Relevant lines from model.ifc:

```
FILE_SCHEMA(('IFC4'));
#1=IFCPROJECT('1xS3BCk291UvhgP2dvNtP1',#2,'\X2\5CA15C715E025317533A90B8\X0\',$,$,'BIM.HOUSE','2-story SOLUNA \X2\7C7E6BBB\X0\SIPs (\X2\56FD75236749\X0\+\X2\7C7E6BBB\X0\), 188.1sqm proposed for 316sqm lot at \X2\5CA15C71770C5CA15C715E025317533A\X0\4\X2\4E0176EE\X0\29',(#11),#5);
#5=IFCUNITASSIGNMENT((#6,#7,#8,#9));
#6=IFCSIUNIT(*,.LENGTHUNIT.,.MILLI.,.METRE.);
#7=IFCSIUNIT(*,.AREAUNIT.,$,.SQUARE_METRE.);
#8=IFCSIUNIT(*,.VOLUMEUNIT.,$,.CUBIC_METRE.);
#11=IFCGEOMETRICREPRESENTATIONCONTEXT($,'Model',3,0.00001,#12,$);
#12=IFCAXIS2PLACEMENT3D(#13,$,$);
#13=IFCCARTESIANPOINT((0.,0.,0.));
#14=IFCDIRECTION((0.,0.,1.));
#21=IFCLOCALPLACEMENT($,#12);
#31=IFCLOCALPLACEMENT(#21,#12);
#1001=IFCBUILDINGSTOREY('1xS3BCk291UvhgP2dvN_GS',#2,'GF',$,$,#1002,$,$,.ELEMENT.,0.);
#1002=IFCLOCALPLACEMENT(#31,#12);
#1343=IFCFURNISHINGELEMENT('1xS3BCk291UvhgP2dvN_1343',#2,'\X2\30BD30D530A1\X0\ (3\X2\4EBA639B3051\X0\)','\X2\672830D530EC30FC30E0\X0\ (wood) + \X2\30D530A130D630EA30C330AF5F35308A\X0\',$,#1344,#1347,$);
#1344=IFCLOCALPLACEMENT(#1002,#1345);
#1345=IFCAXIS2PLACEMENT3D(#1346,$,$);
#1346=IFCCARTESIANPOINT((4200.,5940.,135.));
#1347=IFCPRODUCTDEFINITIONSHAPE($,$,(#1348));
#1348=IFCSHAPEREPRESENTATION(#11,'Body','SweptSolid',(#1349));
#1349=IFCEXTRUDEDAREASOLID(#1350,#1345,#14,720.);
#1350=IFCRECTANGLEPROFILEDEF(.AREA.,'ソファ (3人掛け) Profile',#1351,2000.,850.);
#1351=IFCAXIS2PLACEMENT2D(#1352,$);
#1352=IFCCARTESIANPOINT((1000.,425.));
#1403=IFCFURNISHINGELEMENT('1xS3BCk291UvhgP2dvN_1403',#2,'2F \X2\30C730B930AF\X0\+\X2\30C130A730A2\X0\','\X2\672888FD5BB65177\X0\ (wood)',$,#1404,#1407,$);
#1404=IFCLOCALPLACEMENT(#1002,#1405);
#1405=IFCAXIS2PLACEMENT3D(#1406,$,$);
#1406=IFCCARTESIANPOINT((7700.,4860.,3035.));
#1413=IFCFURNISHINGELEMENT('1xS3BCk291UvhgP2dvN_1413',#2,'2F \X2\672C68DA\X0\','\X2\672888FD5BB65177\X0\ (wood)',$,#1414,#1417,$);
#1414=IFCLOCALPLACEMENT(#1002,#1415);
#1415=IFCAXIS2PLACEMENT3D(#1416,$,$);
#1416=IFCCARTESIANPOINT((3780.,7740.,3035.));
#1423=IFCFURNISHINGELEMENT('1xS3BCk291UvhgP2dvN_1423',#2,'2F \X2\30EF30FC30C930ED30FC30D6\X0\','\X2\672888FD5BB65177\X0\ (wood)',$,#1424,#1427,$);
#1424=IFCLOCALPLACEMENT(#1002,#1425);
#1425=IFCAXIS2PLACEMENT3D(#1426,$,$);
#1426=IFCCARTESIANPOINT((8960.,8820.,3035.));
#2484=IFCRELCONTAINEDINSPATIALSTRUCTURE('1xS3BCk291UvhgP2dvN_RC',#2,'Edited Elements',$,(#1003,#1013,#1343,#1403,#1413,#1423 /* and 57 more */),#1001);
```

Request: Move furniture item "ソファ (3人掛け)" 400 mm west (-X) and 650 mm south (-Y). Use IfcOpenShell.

```python
import ifcopenshell
import ifcopenshell.api.geometry
import ifcopenshell.util.placement
import ifcopenshell.util.unit

model = ifcopenshell.open("model.ifc")
unit_scale = ifcopenshell.util.unit.calculate_unit_scale(model)

item = model.by_id(1343)
matrix = ifcopenshell.util.placement.get_local_placement(item.ObjectPlacement)
matrix[0, 3] -= 0.4 / unit_scale
matrix[1, 3] -= 0.65 / unit_scale
ifcopenshell.api.geometry.edit_object_placement(model, product=item, matrix=matrix, is_si=False)

print(ifcopenshell.util.placement.get_local_placement(item.ObjectPlacement).round(3) + 0.0)

model.write("model_rev.ifc")
```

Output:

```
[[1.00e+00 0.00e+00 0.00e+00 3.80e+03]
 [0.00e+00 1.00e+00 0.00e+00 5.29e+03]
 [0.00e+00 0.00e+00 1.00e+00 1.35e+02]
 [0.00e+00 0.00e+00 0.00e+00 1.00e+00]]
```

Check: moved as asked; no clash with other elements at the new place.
